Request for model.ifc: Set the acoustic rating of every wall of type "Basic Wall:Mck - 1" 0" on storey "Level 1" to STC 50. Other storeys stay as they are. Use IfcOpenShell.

First a look at what the model holds.

```python
import ifcopenshell
import ifcopenshell.util.element

model = ifcopenshell.open("model.ifc")
print(model.schema)
storey = next(s for s in model.by_type("IfcBuildingStorey") if s.Name == "Level 1")
walls = [e for e in ifcopenshell.util.element.get_decomposition(storey) if e.is_a("IfcWall")]
seen = {}
for e in walls:
    element_type = ifcopenshell.util.element.get_type(e)
    key = (element_type.Name if element_type != e and element_type else None, ifcopenshell.util.element.get_pset(e, "Pset_WallCommon", "AcousticRating"))
    seen[key] = seen.get(key, 0) + 1
for (name, value), count in sorted(seen.items(), key=str):
    print(count, "x", name, "|", value)
```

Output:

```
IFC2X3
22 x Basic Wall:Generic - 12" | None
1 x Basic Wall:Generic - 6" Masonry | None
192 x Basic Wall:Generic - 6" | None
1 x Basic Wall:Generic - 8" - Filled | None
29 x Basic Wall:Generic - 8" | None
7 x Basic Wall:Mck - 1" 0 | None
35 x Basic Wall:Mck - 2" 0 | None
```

```python
import ifcopenshell
import ifcopenshell.api.pset
import ifcopenshell.util.element

model = ifcopenshell.open("model.ifc")

storey = next(s for s in model.by_type("IfcBuildingStorey") if s.Name == "Level 1")
walls = [e for e in ifcopenshell.util.element.get_decomposition(storey) if e.is_a("IfcWall")]

count = 0
for e in walls:
    element_type = ifcopenshell.util.element.get_type(e)
    if element_type in (None, e) or element_type.Name != 'Basic Wall:Mck - 1" 0':
        continue
    # add_pset returns the element's existing set when there is one.
    pset = ifcopenshell.api.pset.add_pset(model, product=e, name="Pset_WallCommon")
    ifcopenshell.api.pset.edit_pset(model, pset=pset, properties={"AcousticRating": "STC 50"})
    count += 1

print(count, "walls updated")

model.write("model-out.ifc")
```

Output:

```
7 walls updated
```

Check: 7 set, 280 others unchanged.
